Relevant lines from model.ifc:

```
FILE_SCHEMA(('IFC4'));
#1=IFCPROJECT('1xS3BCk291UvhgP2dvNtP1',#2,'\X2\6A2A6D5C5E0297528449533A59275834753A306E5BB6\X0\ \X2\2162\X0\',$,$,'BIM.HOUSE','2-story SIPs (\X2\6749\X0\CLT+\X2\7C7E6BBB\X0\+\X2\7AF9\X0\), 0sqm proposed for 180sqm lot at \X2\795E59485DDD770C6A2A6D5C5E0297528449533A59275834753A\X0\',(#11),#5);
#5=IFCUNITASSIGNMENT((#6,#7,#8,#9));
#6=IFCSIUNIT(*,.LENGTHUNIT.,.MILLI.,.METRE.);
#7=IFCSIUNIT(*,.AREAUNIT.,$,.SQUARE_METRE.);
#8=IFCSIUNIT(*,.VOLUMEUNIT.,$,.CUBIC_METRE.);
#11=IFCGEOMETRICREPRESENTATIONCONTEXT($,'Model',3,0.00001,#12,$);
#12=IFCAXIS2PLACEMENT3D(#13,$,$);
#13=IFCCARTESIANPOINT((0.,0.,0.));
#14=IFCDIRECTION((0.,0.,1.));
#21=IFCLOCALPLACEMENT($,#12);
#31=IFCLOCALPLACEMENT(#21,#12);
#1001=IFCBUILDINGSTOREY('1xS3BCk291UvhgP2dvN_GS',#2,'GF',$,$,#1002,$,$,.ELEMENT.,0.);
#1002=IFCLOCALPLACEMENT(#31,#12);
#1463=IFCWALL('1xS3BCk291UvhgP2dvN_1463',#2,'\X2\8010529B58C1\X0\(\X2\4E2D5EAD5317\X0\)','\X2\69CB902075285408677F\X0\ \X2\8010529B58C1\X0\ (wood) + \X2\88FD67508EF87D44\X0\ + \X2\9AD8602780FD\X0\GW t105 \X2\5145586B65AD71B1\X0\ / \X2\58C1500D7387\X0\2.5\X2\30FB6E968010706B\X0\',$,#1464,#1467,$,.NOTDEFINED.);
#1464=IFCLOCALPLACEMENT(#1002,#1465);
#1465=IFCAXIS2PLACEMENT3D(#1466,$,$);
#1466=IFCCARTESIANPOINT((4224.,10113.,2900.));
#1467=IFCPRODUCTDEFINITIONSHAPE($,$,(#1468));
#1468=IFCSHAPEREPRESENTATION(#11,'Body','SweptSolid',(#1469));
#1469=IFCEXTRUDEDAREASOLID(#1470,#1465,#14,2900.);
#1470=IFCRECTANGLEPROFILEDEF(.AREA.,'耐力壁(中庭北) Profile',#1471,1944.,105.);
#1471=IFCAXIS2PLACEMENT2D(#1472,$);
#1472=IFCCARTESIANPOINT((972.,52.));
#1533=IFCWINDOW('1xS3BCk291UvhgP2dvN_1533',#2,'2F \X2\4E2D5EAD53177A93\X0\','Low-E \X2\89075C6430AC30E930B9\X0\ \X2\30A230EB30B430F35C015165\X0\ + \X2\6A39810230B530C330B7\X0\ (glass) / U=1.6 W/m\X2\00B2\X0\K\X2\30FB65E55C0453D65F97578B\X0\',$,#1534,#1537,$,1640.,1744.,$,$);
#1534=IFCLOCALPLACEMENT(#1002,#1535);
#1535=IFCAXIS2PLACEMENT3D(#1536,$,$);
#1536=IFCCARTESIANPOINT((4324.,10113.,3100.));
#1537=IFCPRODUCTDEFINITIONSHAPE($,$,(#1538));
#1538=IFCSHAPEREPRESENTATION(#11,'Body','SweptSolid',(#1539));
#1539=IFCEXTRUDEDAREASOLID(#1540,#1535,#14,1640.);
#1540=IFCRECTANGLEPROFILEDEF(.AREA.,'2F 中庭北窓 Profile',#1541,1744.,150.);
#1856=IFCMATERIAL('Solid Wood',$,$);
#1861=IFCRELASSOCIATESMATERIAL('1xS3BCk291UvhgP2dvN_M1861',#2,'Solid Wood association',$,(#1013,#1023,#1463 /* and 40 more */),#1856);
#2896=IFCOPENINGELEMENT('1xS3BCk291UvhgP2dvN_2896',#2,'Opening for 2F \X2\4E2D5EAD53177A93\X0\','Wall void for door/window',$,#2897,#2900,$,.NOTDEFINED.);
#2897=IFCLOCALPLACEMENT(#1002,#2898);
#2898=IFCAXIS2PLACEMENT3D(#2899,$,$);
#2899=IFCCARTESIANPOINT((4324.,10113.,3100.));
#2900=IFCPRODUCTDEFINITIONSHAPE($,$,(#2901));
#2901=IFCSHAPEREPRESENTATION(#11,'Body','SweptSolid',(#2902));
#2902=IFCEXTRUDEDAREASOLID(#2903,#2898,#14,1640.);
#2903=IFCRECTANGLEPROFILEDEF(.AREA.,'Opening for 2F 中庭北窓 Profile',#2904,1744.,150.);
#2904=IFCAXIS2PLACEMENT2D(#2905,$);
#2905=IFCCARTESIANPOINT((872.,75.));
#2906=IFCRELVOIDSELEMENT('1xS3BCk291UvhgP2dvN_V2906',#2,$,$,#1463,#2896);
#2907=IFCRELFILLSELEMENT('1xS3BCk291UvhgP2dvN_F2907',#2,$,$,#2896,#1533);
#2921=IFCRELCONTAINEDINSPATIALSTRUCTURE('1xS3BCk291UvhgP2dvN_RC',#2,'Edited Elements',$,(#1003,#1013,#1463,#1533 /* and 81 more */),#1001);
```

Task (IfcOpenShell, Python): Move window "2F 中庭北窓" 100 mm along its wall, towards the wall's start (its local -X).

```python
import ifcopenshell
import ifcopenshell.api.geometry
import ifcopenshell.util.placement

model = ifcopenshell.open("model.ifc")

window = model.by_guid("1xS3BCk291UvhgP2dvN_1533")
opening = window.FillsVoids[0].RelatingOpeningElement
wall = opening.VoidsElements[0].RelatingBuildingElement

wall_matrix = ifcopenshell.util.placement.get_local_placement(wall.ObjectPlacement)
shift = wall_matrix[:3, 0] * -100.0
before = ifcopenshell.util.placement.get_local_placement(window.ObjectPlacement)[:3, 3].copy()

# The window is not placed relative to its opening, so move both.
for product in (opening, window):
    matrix = ifcopenshell.util.placement.get_local_placement(product.ObjectPlacement)
    matrix[:3, 3] += shift
    ifcopenshell.api.geometry.edit_object_placement(model, product=product, matrix=matrix, is_si=False)

after = ifcopenshell.util.placement.get_local_placement(window.ObjectPlacement)[:3, 3]
print("window moved by", (after - before).round(3) + 0.0)

model.write("model_updated.ifc")
```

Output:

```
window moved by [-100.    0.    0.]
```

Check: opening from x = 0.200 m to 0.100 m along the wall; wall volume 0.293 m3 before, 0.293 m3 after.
